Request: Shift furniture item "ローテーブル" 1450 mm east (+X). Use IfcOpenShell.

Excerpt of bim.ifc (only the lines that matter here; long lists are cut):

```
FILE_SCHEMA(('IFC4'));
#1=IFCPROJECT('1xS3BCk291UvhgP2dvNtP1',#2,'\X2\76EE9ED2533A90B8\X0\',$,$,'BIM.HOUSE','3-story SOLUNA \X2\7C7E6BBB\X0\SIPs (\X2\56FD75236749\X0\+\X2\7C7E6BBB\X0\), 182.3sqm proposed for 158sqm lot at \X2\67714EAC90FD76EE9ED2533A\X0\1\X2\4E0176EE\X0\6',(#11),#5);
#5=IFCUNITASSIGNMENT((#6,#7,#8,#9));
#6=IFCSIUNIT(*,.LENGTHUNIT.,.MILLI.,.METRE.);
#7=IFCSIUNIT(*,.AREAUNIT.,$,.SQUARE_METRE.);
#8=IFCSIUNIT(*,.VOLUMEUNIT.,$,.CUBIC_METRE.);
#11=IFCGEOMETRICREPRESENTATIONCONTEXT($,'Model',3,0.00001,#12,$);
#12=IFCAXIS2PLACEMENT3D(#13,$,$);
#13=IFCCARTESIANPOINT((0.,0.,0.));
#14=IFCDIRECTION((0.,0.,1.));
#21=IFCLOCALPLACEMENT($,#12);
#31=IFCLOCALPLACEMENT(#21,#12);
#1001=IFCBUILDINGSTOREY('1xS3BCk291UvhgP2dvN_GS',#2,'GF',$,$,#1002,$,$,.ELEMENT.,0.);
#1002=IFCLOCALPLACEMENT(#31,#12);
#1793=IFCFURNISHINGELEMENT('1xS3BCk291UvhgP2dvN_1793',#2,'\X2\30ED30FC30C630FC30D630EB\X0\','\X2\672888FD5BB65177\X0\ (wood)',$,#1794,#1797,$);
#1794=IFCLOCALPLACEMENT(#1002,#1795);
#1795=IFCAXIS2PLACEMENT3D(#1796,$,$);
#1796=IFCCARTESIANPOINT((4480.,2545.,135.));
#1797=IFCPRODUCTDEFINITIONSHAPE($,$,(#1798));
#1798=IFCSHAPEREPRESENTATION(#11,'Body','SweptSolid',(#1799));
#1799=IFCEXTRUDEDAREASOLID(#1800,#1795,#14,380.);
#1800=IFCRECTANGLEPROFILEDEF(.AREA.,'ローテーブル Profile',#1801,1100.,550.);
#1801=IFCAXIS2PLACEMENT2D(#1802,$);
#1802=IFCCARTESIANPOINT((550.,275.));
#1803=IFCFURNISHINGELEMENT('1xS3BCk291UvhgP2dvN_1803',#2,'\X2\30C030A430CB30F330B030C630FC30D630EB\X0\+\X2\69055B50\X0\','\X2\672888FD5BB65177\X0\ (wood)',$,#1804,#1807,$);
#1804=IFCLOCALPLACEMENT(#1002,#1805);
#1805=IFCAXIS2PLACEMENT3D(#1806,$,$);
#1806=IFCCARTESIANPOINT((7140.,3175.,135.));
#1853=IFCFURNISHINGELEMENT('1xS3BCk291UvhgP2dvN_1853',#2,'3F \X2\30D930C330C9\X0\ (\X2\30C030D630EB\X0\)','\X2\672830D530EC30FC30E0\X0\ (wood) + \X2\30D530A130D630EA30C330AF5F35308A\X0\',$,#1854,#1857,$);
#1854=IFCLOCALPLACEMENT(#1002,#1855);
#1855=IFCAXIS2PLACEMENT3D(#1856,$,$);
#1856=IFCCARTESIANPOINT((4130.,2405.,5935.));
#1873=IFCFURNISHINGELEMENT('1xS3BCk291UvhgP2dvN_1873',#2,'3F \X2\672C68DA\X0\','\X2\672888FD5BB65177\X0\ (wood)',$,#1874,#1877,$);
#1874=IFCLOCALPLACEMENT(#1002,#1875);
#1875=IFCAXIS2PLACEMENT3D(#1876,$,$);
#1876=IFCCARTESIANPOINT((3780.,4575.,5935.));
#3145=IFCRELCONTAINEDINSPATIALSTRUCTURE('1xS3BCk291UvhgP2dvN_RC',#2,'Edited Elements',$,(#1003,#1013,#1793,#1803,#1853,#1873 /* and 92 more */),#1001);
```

```python
import ifcopenshell
import ifcopenshell.api.geometry
import ifcopenshell.util.placement
import ifcopenshell.util.unit

model = ifcopenshell.open("bim.ifc")
unit_scale = ifcopenshell.util.unit.calculate_unit_scale(model)

item = model.by_guid("1xS3BCk291UvhgP2dvN_1793")
matrix = ifcopenshell.util.placement.get_local_placement(item.ObjectPlacement)
matrix[0, 3] += 1.45 / unit_scale
ifcopenshell.api.geometry.edit_object_placement(model, product=item, matrix=matrix, is_si=False)

print(ifcopenshell.util.placement.get_local_placement(item.ObjectPlacement).round(3) + 0.0)

model.write("bim-out.ifc")
```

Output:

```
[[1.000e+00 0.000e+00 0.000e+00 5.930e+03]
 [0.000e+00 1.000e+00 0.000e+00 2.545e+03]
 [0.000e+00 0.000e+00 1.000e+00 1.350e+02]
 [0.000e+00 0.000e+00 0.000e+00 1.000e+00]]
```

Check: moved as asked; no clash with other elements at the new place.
